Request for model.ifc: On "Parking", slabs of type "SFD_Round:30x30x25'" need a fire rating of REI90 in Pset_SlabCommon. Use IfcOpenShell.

First a look at what the model holds.

```python
import ifcopenshell
import ifcopenshell.util.element

model = ifcopenshell.open("model.ifc")
print(model.schema)
storey = next(s for s in model.by_type("IfcBuildingStorey") if s.Name == "Parking")
slabs = [e for e in ifcopenshell.util.element.get_decomposition(storey) if e.is_a("IfcSlab")]
seen = {}
for e in slabs:
    element_type = ifcopenshell.util.element.get_type(e)
    key = (element_type.Name if element_type != e and element_type else None, ifcopenshell.util.element.get_pset(e, "Pset_SlabCommon", "FireRating"))
    seen[key] = seen.get(key, 0) + 1
for (name, value), count in sorted(seen.items(), key=str):
    print(count, "x", name, "|", value)
```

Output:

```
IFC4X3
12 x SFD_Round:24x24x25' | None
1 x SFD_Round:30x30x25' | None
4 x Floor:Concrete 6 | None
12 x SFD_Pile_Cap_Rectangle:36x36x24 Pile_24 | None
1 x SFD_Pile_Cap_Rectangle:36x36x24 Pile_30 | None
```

```python
import ifcopenshell
import ifcopenshell.api.pset
import ifcopenshell.util.element

model = ifcopenshell.open("model.ifc")

storey = next(s for s in model.by_type("IfcBuildingStorey") if s.Name == "Parking")
slabs = [e for e in ifcopenshell.util.element.get_decomposition(storey) if e.is_a("IfcSlab")]

count = 0
for e in slabs:
    element_type = ifcopenshell.util.element.get_type(e)
    if element_type in (None, e) or element_type.Name != "SFD_Round:30x30x25'":
        continue
    # add_pset returns the element's existing set when there is one.
    pset = ifcopenshell.api.pset.add_pset(model, product=e, name="Pset_SlabCommon")
    ifcopenshell.api.pset.edit_pset(model, pset=pset, properties={"FireRating": "REI90"})
    count += 1

print(count, "slabs updated")

model.write("model_rev.ifc")
```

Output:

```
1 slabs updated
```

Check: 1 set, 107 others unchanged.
